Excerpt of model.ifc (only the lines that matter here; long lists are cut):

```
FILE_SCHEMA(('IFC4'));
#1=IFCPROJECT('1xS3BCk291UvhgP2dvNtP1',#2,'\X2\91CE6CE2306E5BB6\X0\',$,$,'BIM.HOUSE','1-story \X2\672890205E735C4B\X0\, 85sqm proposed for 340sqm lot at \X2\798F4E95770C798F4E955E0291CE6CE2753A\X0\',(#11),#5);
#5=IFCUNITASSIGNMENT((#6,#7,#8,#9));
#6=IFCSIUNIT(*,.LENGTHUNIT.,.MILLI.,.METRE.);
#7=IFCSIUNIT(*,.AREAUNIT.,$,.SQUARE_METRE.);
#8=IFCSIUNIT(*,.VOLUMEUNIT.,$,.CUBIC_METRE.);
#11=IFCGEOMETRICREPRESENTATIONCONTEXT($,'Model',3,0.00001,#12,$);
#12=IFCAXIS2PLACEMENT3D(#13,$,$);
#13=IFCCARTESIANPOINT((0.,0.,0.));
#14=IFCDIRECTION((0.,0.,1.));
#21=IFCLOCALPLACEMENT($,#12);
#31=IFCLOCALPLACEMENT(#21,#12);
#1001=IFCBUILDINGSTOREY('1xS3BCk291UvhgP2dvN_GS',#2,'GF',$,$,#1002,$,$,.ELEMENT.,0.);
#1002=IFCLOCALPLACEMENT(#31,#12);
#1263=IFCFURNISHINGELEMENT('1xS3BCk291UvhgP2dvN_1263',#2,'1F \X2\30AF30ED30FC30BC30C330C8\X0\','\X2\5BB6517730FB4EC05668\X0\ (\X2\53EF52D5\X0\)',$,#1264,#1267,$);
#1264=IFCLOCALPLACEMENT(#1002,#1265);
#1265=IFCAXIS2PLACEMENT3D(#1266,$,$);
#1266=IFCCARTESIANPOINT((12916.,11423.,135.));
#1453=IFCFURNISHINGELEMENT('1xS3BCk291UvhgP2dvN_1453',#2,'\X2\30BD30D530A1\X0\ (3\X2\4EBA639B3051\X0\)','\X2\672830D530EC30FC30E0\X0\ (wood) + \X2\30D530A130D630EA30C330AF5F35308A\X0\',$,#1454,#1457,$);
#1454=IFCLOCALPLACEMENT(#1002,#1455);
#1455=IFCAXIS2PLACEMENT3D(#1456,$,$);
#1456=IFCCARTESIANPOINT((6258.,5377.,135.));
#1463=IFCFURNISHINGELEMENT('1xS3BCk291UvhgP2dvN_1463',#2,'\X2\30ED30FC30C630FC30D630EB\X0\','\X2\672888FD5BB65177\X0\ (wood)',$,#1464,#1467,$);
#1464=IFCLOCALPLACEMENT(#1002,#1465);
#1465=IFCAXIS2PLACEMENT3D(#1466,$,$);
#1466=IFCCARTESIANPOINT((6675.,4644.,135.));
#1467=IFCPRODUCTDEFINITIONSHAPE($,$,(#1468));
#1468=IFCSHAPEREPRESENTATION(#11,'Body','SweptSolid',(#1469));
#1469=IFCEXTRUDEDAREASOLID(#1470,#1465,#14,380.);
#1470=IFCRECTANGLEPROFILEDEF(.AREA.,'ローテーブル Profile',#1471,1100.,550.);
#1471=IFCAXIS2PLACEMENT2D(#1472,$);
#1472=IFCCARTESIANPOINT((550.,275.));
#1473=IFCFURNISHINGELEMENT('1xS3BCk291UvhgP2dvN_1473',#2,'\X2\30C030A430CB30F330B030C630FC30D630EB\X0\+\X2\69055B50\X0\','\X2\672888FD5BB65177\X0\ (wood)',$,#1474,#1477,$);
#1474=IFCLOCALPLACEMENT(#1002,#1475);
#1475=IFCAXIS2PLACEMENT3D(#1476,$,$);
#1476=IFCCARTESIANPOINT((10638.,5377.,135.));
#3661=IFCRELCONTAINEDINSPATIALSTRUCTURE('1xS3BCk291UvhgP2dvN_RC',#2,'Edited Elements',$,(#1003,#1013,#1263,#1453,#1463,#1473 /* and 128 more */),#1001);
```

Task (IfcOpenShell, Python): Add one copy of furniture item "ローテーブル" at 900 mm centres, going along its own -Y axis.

```python
import ifcopenshell
import ifcopenshell.api.geometry
import ifcopenshell.api.root
import ifcopenshell.util.element
import ifcopenshell.util.placement
import ifcopenshell.util.unit

model = ifcopenshell.open("model.ifc")
unit_scale = ifcopenshell.util.unit.calculate_unit_scale(model)


def reuse_history(source, copy):
    """copy_class also copies each property set's owner history, people and application; keep the originals."""
    for rel in copy.IsDefinedBy:
        if rel.is_a("IfcRelDefinesByProperties") and (history := rel.RelatingPropertyDefinition.OwnerHistory):
            rel.RelatingPropertyDefinition.OwnerHistory = source.OwnerHistory
            ifcopenshell.util.element.remove_deep2(model, history)


source = model.by_guid("1xS3BCk291UvhgP2dvN_1463")
base = ifcopenshell.util.placement.get_local_placement(source.ObjectPlacement)
step = -base[:3, 1] * 0.9 / unit_scale

for i in range(1, 2):
    copy = ifcopenshell.api.root.copy_class(model, product=source)
    copy.Representation = ifcopenshell.util.element.copy_deep(
        model, source.Representation, exclude=["IfcGeometricRepresentationContext", "IfcRepresentationMap"]
    )
    reuse_history(source, copy)
    matrix = base.copy()
    matrix[:3, 3] += i * step
    print("added at", matrix[:3, 3].round(3) + 0.0)
    ifcopenshell.api.geometry.edit_object_placement(model, product=copy, matrix=matrix, is_si=False)

model.write("model-out.ifc")
```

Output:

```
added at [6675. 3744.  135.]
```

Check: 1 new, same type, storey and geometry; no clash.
